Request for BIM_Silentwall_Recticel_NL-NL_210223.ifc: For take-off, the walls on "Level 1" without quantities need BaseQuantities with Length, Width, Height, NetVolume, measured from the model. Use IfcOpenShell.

First a look at what the model holds.

```python
import ifcopenshell
import ifcopenshell.util.element
import ifcopenshell.util.unit

model = ifcopenshell.open("BIM_Silentwall_Recticel_NL-NL_210223.ifc")
print(model.schema)
for unit_type in ("LENGTHUNIT", "AREAUNIT", "VOLUMEUNIT"):
    print(unit_type, ifcopenshell.util.unit.calculate_unit_scale(model, unit_type))
storey = next(s for s in model.by_type("IfcBuildingStorey") if s.Name == "Level 1")
walls = [e for e in ifcopenshell.util.element.get_decomposition(storey) if e.is_a("IfcWall")]
for e in sorted(walls, key=lambda e: e.id()):
    print(e.id(), e.is_a(), e.Name, list(ifcopenshell.util.element.get_psets(e, qtos_only=True)), sep=" | ")
```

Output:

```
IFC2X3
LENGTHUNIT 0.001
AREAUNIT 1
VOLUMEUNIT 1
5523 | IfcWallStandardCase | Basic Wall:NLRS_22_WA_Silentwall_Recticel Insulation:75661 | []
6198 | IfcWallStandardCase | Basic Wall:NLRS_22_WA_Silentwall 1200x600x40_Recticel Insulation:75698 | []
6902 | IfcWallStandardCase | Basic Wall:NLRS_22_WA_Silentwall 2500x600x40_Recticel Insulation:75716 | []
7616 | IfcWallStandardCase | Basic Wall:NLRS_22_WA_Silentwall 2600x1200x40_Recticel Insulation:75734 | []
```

```python
import ifcopenshell
import ifcopenshell.api.pset
import ifcopenshell.geom
import ifcopenshell.util.element
import ifcopenshell.util.shape
import ifcopenshell.util.unit

model = ifcopenshell.open("BIM_Silentwall_Recticel_NL-NL_210223.ifc")
unit_scale = ifcopenshell.util.unit.calculate_unit_scale(model)
volume_scale = ifcopenshell.util.unit.calculate_unit_scale(model, "VOLUMEUNIT")
settings = ifcopenshell.geom.settings()

storey = next(s for s in model.by_type("IfcBuildingStorey") if s.Name == "Level 1")
walls = [e for e in ifcopenshell.util.element.get_decomposition(storey) if e.is_a("IfcWall")]

for e in sorted(walls, key=lambda e: e.id()):
    if ifcopenshell.util.element.get_psets(e, qtos_only=True, should_inherit=False):
        continue
    # Geometry comes back in metres, in the element's own axes.
    shape = ifcopenshell.geom.create_shape(settings, e)
    values = {
        "Length": ifcopenshell.util.shape.get_x(shape.geometry) / unit_scale,
        "Width": ifcopenshell.util.shape.get_y(shape.geometry) / unit_scale,
        "Height": ifcopenshell.util.shape.get_z(shape.geometry) / unit_scale,
        "NetVolume": ifcopenshell.util.shape.get_volume(shape.geometry) / volume_scale,
    }
    qto = ifcopenshell.api.pset.add_qto(model, product=e, name="BaseQuantities")
    ifcopenshell.api.pset.edit_qto(model, qto=qto, properties=values)
    print(e.id(), {k: round(v, 3) for k, v in values.items()})

model.write("BIM_Silentwall_Recticel_NL-NL_210223_v2.ifc")
```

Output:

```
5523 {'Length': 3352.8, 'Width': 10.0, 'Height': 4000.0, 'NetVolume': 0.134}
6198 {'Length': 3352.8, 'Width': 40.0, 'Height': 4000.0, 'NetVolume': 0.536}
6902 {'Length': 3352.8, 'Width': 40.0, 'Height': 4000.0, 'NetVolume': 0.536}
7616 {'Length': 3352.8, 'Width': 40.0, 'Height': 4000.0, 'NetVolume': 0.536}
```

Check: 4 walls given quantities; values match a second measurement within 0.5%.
